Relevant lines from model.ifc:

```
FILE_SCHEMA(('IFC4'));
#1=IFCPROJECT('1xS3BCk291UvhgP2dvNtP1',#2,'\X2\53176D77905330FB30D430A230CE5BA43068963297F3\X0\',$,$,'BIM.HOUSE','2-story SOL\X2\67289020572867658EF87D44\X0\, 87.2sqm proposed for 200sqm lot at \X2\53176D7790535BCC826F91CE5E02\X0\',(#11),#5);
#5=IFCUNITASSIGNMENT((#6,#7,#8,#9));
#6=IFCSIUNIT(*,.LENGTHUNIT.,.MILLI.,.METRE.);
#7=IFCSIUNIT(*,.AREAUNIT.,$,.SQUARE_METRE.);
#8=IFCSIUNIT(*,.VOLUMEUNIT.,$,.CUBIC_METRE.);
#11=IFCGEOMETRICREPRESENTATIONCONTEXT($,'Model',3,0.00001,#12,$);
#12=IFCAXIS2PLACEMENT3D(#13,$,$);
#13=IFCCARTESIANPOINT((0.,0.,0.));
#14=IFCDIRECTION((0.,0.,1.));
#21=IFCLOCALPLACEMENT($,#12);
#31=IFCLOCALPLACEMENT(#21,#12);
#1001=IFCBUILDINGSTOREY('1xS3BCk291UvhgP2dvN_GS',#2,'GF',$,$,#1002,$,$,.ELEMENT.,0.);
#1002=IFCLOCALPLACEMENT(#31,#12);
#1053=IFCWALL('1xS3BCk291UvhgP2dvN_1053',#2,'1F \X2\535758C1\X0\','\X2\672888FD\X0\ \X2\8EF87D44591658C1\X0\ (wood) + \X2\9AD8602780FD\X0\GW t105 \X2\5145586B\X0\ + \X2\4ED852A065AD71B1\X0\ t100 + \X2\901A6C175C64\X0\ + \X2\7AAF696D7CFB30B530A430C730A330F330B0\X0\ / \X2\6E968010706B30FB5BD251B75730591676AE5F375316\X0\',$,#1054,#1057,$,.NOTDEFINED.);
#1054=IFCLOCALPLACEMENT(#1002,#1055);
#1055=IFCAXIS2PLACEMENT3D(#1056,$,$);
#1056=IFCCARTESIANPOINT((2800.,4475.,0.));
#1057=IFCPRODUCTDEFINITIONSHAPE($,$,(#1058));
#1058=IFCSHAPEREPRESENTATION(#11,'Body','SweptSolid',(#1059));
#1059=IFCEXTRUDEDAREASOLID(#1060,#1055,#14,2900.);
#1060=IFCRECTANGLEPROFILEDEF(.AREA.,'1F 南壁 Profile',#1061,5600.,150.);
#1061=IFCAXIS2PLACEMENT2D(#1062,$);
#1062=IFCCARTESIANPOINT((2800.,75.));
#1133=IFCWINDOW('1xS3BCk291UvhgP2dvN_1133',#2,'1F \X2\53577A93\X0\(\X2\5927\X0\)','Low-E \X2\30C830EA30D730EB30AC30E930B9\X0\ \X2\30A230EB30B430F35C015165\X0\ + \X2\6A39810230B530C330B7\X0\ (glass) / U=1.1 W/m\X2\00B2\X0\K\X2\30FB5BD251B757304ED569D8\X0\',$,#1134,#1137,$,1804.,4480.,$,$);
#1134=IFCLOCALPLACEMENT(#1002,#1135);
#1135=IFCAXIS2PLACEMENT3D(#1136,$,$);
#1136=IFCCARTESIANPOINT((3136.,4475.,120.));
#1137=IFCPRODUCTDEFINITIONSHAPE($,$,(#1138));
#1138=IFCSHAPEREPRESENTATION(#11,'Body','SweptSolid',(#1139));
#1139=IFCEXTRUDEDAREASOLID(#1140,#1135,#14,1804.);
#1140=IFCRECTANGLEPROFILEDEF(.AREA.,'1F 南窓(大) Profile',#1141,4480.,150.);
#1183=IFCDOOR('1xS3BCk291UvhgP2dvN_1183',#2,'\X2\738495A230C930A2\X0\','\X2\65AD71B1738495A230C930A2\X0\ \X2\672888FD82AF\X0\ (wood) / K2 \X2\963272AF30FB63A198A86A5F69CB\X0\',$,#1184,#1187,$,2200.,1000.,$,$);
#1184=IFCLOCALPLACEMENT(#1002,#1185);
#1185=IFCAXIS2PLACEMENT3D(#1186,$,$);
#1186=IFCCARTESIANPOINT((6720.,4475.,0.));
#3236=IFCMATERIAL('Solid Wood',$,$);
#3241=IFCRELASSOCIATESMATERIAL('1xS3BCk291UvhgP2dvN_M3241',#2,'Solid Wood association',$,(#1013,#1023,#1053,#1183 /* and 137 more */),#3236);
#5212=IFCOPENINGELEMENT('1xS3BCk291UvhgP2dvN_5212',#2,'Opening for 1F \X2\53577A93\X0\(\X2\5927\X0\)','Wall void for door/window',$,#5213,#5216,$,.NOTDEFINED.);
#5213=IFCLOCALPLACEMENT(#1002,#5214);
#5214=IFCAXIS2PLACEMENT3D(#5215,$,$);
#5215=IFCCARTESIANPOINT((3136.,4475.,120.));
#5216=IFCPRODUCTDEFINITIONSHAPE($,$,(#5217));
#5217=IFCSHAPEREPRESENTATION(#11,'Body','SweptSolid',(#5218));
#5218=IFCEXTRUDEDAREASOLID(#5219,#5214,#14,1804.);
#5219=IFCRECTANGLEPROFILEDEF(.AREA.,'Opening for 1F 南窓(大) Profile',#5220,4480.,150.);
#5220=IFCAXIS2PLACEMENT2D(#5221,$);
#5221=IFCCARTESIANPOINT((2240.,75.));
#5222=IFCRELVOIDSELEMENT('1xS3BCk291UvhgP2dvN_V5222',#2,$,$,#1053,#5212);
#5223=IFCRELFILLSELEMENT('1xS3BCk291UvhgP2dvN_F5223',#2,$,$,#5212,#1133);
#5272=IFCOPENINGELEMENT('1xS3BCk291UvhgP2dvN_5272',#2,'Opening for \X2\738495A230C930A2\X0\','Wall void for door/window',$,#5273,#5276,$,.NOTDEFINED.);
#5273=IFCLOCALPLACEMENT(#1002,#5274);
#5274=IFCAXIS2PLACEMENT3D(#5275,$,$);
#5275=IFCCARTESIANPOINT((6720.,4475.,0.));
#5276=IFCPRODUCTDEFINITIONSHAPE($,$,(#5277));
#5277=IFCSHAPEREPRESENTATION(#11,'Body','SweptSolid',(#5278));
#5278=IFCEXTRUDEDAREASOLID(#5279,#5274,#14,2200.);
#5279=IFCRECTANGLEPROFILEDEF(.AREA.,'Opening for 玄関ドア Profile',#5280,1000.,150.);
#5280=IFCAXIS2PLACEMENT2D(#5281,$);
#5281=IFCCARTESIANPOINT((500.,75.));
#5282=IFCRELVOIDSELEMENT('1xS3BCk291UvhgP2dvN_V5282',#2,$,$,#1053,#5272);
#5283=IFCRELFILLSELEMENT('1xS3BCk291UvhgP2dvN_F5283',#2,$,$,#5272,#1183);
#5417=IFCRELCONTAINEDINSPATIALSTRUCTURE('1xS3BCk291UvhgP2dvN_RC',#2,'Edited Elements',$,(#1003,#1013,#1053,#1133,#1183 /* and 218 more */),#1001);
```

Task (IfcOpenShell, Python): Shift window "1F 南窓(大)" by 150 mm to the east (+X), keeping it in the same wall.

```python
import ifcopenshell
import ifcopenshell.api.geometry
import ifcopenshell.util.placement

model = ifcopenshell.open("model.ifc")

window = model.by_id(1133)
opening = window.FillsVoids[0].RelatingOpeningElement
wall = opening.VoidsElements[0].RelatingBuildingElement

wall_matrix = ifcopenshell.util.placement.get_local_placement(wall.ObjectPlacement)
shift = wall_matrix[:3, 0] * 150.0
before = ifcopenshell.util.placement.get_local_placement(window.ObjectPlacement)[:3, 3].copy()

# The window is not placed relative to its opening, so move both.
for product in (opening, window):
    matrix = ifcopenshell.util.placement.get_local_placement(product.ObjectPlacement)
    matrix[:3, 3] += shift
    ifcopenshell.api.geometry.edit_object_placement(model, product=product, matrix=matrix, is_si=False)

after = ifcopenshell.util.placement.get_local_placement(window.ObjectPlacement)[:3, 3]
print("window moved by", (after - before).round(3) + 0.0)

model.write("model_edited.ifc")
```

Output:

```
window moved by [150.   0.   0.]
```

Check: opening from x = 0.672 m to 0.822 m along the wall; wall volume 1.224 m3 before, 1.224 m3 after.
